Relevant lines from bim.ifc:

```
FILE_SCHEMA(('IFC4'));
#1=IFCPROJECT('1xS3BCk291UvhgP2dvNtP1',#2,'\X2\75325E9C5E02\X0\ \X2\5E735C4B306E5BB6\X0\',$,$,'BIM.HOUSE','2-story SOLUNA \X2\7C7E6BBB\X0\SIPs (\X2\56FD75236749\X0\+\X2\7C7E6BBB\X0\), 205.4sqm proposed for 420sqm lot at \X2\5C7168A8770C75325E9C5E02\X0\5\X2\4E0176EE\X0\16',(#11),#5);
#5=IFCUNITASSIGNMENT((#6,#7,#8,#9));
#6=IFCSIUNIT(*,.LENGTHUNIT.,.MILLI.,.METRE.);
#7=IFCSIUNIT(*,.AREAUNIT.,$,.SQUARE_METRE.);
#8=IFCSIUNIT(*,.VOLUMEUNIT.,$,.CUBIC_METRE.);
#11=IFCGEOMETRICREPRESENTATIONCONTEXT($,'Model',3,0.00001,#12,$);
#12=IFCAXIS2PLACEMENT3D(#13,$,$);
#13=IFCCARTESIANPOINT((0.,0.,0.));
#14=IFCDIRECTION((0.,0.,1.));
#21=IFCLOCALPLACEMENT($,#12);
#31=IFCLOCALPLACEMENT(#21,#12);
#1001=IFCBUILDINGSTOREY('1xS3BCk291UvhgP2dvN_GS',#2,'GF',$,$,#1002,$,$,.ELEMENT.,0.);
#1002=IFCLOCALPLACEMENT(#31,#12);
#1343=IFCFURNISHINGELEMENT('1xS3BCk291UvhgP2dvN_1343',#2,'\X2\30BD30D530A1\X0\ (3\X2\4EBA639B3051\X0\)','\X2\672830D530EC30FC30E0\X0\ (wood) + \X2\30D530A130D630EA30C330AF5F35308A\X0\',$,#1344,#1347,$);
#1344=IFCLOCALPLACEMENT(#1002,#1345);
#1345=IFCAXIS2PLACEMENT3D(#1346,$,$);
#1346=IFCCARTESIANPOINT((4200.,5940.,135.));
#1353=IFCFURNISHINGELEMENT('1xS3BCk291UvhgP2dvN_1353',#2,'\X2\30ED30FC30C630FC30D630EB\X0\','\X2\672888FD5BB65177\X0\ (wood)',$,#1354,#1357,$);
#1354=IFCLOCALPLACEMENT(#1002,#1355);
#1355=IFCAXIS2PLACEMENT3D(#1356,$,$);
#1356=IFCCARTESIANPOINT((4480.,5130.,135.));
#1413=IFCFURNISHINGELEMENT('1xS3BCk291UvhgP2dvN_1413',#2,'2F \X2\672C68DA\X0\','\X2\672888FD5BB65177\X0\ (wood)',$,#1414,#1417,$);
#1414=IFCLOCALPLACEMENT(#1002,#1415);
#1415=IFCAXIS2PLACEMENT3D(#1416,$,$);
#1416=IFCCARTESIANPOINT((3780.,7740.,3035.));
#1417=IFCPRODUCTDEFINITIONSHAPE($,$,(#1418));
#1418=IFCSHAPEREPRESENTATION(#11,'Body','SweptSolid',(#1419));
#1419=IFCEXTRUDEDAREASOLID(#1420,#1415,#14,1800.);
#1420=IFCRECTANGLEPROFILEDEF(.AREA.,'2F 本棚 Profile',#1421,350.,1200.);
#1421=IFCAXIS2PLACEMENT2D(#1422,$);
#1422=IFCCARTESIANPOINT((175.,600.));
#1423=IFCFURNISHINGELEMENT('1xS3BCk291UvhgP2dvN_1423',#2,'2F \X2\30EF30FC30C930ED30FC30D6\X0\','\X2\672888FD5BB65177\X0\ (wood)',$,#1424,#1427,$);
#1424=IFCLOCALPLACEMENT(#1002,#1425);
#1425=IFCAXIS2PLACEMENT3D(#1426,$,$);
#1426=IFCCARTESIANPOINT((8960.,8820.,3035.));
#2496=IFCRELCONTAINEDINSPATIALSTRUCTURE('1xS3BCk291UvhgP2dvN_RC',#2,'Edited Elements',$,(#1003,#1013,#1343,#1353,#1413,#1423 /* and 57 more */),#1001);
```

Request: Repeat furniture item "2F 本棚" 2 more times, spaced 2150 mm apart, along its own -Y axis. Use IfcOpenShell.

```python
import ifcopenshell
import ifcopenshell.api.geometry
import ifcopenshell.api.root
import ifcopenshell.util.element
import ifcopenshell.util.placement
import ifcopenshell.util.unit

model = ifcopenshell.open("bim.ifc")
unit_scale = ifcopenshell.util.unit.calculate_unit_scale(model)


def reuse_history(source, copy):
    """copy_class also copies each property set's owner history, people and application; keep the originals."""
    for rel in copy.IsDefinedBy:
        if rel.is_a("IfcRelDefinesByProperties") and (history := rel.RelatingPropertyDefinition.OwnerHistory):
            rel.RelatingPropertyDefinition.OwnerHistory = source.OwnerHistory
            ifcopenshell.util.element.remove_deep2(model, history)


source = model.by_guid("1xS3BCk291UvhgP2dvN_1413")
base = ifcopenshell.util.placement.get_local_placement(source.ObjectPlacement)
step = -base[:3, 1] * 2.15 / unit_scale

for i in range(1, 3):
    copy = ifcopenshell.api.root.copy_class(model, product=source)
    copy.Representation = ifcopenshell.util.element.copy_deep(
        model, source.Representation, exclude=["IfcGeometricRepresentationContext", "IfcRepresentationMap"]
    )
    reuse_history(source, copy)
    matrix = base.copy()
    matrix[:3, 3] += i * step
    print("added at", matrix[:3, 3].round(3) + 0.0)
    ifcopenshell.api.geometry.edit_object_placement(model, product=copy, matrix=matrix, is_si=False)

model.write("bim-out.ifc")
```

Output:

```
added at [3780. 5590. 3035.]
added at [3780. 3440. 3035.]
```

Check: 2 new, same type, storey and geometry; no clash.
